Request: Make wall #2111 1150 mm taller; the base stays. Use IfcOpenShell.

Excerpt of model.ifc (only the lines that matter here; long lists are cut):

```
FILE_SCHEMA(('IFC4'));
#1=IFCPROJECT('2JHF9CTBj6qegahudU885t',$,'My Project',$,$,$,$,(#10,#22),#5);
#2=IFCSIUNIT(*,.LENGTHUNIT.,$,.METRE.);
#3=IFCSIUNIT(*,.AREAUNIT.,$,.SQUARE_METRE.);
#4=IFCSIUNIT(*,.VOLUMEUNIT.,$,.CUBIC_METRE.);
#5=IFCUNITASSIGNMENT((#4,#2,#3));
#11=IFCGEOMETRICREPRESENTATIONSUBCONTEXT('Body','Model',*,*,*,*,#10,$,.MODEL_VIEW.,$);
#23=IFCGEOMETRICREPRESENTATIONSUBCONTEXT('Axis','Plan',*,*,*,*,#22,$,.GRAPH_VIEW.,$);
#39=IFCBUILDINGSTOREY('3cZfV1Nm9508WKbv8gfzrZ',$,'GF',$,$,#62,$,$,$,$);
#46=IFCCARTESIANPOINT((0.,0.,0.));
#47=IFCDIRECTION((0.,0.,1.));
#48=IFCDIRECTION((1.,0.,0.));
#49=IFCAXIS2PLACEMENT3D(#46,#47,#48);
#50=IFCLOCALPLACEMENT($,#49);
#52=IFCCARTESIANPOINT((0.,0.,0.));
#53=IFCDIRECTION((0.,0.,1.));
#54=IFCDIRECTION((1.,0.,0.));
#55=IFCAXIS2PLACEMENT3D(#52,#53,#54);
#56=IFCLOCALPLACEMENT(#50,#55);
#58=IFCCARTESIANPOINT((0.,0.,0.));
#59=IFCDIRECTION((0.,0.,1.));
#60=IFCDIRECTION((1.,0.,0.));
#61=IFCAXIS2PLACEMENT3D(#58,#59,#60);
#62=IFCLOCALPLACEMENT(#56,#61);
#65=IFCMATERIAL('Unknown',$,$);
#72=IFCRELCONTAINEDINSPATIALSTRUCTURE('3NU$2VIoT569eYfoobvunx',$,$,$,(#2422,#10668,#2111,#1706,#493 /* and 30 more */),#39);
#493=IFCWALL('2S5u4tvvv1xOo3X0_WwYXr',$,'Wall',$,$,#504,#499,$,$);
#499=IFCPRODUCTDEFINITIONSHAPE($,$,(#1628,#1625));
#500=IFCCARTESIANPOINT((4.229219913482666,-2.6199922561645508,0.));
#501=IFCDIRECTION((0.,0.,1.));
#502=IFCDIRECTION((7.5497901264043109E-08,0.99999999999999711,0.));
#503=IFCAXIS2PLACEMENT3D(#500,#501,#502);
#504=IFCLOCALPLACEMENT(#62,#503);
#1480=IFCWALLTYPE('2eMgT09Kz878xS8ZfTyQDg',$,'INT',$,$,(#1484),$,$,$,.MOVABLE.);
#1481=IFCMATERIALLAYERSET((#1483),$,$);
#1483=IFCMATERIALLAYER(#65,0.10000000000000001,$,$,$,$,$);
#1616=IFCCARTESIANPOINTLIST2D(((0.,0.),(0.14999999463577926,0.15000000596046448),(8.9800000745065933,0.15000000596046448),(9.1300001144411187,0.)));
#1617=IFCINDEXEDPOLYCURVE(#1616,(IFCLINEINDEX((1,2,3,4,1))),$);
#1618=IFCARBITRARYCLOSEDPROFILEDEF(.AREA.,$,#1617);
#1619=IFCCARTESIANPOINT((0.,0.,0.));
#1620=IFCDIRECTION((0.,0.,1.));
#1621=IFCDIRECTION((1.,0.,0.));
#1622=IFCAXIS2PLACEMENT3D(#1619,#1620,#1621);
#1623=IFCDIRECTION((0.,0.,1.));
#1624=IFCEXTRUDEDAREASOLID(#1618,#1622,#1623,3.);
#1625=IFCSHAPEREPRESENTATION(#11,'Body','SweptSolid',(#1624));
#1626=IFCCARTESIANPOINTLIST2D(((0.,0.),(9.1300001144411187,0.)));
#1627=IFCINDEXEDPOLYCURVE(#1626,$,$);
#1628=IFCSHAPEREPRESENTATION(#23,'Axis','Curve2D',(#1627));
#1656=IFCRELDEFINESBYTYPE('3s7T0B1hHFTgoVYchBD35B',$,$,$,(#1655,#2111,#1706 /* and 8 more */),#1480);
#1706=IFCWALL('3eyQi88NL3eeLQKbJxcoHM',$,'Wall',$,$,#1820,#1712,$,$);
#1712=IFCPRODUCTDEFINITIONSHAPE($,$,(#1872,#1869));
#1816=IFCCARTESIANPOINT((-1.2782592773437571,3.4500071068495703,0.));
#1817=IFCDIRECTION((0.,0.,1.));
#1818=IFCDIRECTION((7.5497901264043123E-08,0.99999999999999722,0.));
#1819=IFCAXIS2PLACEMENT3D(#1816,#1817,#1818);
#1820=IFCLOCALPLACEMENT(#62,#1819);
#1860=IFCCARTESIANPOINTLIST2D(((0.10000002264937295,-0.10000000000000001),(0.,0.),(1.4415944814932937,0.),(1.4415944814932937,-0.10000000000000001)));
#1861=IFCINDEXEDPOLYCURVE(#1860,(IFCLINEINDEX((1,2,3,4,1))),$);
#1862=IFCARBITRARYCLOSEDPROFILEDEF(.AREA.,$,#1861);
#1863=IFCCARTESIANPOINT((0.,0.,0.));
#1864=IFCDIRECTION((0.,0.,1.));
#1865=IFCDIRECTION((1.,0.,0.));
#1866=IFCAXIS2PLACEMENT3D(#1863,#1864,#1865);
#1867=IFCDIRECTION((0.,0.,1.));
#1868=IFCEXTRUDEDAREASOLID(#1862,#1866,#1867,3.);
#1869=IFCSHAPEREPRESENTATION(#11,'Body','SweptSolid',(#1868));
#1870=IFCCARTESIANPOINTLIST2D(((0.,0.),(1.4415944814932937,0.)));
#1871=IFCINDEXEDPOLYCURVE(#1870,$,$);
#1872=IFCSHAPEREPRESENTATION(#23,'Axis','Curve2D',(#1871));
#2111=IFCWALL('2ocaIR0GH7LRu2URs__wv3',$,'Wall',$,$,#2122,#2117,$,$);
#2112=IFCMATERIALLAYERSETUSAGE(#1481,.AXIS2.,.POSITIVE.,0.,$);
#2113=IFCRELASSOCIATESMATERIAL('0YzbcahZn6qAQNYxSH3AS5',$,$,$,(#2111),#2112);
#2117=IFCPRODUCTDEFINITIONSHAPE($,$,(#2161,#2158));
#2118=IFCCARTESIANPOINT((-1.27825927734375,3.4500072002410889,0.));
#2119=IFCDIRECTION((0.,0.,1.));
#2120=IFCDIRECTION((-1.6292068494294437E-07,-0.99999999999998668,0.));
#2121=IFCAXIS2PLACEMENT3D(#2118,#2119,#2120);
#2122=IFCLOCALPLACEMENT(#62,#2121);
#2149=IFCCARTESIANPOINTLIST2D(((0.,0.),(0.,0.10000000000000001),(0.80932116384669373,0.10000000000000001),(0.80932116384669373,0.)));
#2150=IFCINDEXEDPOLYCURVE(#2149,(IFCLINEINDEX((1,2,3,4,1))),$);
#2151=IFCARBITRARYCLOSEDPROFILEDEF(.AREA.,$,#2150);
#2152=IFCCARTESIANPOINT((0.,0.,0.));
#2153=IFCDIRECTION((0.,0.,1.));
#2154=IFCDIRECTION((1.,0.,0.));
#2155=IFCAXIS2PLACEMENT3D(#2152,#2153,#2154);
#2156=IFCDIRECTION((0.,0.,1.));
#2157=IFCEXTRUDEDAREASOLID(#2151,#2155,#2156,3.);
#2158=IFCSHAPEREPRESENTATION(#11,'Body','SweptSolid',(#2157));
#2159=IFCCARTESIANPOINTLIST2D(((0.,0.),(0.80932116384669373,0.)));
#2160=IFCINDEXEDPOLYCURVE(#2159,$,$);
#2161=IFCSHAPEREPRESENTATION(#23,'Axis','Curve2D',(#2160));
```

```python
import ifcopenshell
import ifcopenshell.geom
import ifcopenshell.util.representation
import ifcopenshell.util.shape
import ifcopenshell.util.unit

model = ifcopenshell.open("model.ifc")
unit_scale = ifcopenshell.util.unit.calculate_unit_scale(model)
settings = ifcopenshell.geom.settings()


def volume(element):
    """Net volume in cubic metres, openings subtracted."""
    shape = ifcopenshell.geom.create_shape(settings, element)
    return ifcopenshell.util.shape.get_volume(shape.geometry)


wall = model.by_guid("2ocaIR0GH7LRu2URs__wv3")
before = volume(wall)

body = ifcopenshell.util.representation.get_representation(wall, "Model", "Body")
solid = body.Items[0]
old_height = solid.Depth
solid.Depth += 1.15 / unit_scale
after = volume(wall)

print(f"height {old_height:g} -> {solid.Depth:g}, volume {before:.3f} -> {after:.3f} m3")

model.write("model-out.ifc")
```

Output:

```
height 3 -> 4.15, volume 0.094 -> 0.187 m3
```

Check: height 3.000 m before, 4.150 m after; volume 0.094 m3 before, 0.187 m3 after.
